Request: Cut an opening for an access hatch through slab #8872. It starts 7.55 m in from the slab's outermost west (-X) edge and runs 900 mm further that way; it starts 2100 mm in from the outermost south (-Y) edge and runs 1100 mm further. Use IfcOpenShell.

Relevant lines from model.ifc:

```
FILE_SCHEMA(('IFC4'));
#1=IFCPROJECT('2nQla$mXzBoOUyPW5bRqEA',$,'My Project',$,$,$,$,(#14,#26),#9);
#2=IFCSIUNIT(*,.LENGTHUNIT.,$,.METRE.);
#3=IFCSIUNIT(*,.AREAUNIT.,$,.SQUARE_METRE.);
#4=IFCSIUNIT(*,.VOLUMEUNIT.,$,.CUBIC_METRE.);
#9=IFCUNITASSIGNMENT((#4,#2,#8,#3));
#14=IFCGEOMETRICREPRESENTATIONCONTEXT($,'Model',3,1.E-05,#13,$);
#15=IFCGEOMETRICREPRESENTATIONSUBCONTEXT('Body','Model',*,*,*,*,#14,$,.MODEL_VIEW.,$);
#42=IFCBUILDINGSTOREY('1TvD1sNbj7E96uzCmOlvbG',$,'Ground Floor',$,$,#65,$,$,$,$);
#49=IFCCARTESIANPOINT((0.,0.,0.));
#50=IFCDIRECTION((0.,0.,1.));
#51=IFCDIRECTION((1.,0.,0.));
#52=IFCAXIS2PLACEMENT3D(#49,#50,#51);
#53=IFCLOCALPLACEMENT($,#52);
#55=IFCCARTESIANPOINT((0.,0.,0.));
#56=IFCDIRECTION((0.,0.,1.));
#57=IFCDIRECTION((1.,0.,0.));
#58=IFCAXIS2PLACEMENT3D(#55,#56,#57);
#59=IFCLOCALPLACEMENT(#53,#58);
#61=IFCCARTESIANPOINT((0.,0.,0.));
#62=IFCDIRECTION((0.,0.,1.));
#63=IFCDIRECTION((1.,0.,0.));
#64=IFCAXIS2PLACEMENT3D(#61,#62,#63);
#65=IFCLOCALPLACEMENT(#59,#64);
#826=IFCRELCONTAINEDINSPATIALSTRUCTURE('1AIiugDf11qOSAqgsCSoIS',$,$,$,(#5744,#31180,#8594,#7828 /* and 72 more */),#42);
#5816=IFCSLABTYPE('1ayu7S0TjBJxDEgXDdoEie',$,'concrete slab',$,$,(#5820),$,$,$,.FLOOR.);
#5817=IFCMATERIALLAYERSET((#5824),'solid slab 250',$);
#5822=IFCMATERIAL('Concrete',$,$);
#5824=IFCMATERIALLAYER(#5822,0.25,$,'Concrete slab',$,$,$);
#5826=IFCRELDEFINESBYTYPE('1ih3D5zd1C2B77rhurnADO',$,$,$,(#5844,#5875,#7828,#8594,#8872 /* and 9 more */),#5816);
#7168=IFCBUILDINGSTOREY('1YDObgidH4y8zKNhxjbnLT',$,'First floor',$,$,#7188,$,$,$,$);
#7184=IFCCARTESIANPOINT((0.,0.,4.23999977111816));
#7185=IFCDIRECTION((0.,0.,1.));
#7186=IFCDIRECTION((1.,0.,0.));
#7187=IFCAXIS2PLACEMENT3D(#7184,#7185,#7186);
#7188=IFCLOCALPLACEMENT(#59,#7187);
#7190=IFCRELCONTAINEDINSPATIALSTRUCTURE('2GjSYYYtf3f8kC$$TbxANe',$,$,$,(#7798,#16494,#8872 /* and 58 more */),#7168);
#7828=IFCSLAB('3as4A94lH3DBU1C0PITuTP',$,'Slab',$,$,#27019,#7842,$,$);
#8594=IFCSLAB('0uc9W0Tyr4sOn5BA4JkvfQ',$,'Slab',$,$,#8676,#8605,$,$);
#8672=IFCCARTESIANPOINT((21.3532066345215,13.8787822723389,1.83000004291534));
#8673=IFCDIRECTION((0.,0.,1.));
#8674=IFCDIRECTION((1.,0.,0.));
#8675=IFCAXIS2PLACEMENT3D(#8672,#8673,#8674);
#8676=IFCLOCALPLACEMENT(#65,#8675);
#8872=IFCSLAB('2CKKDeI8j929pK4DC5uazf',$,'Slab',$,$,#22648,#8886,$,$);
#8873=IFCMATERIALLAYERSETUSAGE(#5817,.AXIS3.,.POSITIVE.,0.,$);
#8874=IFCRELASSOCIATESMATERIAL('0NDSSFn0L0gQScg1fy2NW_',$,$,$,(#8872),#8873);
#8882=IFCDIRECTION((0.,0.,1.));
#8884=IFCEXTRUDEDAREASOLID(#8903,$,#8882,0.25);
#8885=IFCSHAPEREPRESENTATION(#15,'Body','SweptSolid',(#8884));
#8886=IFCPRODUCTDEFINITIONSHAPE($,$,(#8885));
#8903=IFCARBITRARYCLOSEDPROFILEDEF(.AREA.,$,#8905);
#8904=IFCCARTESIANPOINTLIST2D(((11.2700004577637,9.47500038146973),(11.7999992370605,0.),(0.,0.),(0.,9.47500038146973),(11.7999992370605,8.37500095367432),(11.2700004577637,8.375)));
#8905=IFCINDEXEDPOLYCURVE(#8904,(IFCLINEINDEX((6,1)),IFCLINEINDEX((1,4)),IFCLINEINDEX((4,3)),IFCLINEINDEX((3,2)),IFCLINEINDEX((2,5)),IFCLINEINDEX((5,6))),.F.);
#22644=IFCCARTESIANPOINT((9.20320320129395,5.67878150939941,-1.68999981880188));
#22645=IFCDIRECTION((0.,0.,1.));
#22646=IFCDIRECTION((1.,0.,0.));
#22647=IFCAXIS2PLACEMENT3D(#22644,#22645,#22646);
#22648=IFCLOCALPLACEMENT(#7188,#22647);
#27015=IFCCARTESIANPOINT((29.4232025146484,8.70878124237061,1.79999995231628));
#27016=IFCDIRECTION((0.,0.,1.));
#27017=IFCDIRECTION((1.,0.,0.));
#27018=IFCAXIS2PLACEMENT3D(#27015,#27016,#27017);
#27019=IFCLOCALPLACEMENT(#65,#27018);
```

```python
import numpy as np
import ifcopenshell
import ifcopenshell.api.feature
import ifcopenshell.api.geometry
import ifcopenshell.api.root
import ifcopenshell.geom
import ifcopenshell.util.placement
import ifcopenshell.util.representation
import ifcopenshell.util.shape
import ifcopenshell.util.unit

model = ifcopenshell.open("model.ifc")
unit_scale = ifcopenshell.util.unit.calculate_unit_scale(model)
settings = ifcopenshell.geom.settings()


def volume(element):
    """Net volume in cubic metres, openings subtracted."""
    shape = ifcopenshell.geom.create_shape(settings, element)
    return ifcopenshell.util.shape.get_volume(shape.geometry)


slab = model.by_id(8872)
before = volume(slab)

# Extent in the slab's own axes, in metres. The edges named are its -X and -Y sides.
slab_shape = ifcopenshell.geom.create_shape(settings, slab)
vertices = ifcopenshell.util.shape.get_vertices(slab_shape.geometry)
x_min, y_min, bottom = vertices.min(axis=0)
top = vertices[:, 2].max()

opening = ifcopenshell.api.root.create_entity(model, ifc_class="IfcOpeningElement", name="Access hatch opening", predefined_type="OPENING")
context = ifcopenshell.util.representation.get_context(model, "Model", "Body", "MODEL_VIEW")
width, depth = 0.9, 1.1
outline = [(0.0, 0.0), (width, 0.0), (width, depth), (0.0, depth), (0.0, 0.0)]
# Overshoot both faces by 50 mm so the cut is clean.
shape = ifcopenshell.api.geometry.add_slab_representation(
    model, context=context, depth=top - bottom + 0.1, polyline=outline
)
ifcopenshell.api.geometry.assign_representation(model, product=opening, representation=shape)

matrix = ifcopenshell.util.placement.get_local_placement(slab.ObjectPlacement)
matrix[:, 3] = matrix @ np.append(np.array([x_min + 7.55, y_min + 2.1, bottom - 0.05]) / unit_scale, 1.0)
ifcopenshell.api.geometry.edit_object_placement(model, product=opening, matrix=matrix, is_si=False)
ifcopenshell.api.feature.add_feature(model, feature=opening, element=slab)

after = volume(slab)

print(f"slab volume {before:.3f} -> {after:.3f} m3")

model.write("model-out.ifc")
```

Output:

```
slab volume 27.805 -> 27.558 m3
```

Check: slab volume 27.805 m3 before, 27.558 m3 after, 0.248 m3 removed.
